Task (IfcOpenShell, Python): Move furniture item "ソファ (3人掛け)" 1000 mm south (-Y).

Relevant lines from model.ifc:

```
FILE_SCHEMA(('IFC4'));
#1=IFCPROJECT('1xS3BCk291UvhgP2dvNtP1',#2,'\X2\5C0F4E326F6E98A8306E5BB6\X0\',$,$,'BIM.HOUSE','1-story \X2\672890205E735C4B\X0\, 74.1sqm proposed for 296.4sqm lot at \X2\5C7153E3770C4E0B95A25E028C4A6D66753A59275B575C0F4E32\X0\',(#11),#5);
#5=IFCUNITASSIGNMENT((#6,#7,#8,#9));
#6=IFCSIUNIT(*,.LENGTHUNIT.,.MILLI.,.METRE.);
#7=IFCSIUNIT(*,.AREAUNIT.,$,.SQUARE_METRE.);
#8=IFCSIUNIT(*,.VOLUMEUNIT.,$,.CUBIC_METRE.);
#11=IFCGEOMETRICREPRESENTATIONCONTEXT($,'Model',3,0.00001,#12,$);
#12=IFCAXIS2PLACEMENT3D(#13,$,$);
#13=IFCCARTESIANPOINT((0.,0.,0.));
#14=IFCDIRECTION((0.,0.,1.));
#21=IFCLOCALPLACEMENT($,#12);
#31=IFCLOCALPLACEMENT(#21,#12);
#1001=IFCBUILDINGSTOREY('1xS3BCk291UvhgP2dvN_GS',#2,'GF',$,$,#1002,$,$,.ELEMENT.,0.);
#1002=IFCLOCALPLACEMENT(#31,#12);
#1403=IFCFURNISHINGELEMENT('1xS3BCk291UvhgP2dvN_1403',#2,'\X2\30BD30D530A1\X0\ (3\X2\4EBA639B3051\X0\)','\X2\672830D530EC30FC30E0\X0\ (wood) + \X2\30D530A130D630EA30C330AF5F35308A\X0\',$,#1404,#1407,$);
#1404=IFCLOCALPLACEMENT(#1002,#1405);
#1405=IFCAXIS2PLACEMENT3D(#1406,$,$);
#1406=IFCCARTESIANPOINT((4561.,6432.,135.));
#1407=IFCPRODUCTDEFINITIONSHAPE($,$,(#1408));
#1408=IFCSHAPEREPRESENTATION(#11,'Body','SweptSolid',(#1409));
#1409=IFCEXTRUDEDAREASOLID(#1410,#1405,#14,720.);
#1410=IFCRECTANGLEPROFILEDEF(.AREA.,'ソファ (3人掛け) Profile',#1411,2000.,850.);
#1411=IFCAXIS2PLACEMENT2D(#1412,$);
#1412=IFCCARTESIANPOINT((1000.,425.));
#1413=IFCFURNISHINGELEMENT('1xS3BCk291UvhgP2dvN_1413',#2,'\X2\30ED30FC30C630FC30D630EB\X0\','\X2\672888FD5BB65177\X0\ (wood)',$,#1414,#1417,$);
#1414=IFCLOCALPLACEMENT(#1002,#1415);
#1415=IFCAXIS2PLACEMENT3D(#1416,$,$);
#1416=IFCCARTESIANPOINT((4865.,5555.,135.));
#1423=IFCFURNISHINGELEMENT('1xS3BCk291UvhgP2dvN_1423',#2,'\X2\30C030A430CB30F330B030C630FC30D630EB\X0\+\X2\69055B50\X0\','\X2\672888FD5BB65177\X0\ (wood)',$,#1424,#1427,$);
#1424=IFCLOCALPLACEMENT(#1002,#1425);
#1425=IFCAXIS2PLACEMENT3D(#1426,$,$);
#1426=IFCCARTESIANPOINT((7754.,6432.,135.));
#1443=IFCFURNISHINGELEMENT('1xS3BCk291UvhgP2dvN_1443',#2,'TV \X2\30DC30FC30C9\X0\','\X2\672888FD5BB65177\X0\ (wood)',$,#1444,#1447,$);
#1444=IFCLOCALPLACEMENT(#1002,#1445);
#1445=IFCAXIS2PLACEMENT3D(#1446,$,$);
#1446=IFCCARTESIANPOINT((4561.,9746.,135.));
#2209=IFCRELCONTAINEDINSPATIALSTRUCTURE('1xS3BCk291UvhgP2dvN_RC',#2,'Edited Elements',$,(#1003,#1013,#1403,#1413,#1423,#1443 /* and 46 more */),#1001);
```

```python
import ifcopenshell
import ifcopenshell.api.geometry
import ifcopenshell.util.placement
import ifcopenshell.util.unit

model = ifcopenshell.open("model.ifc")
unit_scale = ifcopenshell.util.unit.calculate_unit_scale(model)

item = model.by_guid("1xS3BCk291UvhgP2dvN_1403")
matrix = ifcopenshell.util.placement.get_local_placement(item.ObjectPlacement)
matrix[1, 3] -= 1 / unit_scale
ifcopenshell.api.geometry.edit_object_placement(model, product=item, matrix=matrix, is_si=False)

print(ifcopenshell.util.placement.get_local_placement(item.ObjectPlacement).round(3) + 0.0)

model.write("model_updated.ifc")
```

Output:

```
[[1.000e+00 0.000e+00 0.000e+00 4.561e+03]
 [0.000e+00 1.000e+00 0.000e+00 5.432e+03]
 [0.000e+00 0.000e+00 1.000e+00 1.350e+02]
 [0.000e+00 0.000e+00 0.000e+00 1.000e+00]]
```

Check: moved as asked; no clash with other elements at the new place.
